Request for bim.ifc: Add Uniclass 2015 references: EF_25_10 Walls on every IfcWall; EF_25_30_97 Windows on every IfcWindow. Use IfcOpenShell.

First a look at what the model holds.

```python
import ifcopenshell

model = ifcopenshell.open("bim.ifc")
print(model.schema)
print("classifications:", [c.Name for c in model.by_type("IfcClassification")])
for ifc_class in ("IfcDoor", "IfcRoof", "IfcStair", "IfcWall", "IfcWindow"):
    print(ifc_class, len(model.by_type(ifc_class)))
```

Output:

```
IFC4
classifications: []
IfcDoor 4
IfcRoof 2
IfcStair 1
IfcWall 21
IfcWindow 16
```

```python
import ifcopenshell
import ifcopenshell.api.classification

model = ifcopenshell.open("bim.ifc")

system = ifcopenshell.api.classification.add_classification(model, classification="Uniclass 2015")

codes = {
    "IfcWall": ("EF_25_10", "Walls"),
    "IfcWindow": ("EF_25_30_97", "Windows"),
}
for ifc_class, (code, name) in codes.items():
    products = model.by_type(ifc_class)
    ifcopenshell.api.classification.add_reference(
        model, products=products, classification=system, identification=code, name=name
    )
    print(code, len(products))

model.write("bim_v2.ifc")
```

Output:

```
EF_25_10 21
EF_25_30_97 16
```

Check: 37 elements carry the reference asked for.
